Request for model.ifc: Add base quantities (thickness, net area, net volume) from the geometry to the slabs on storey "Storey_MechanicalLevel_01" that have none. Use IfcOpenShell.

First a look at what the model holds.

```python
import ifcopenshell
import ifcopenshell.util.element
import ifcopenshell.util.unit

model = ifcopenshell.open("model.ifc")
print(model.schema)
for unit_type in ("LENGTHUNIT", "AREAUNIT", "VOLUMEUNIT"):
    print(unit_type, ifcopenshell.util.unit.calculate_unit_scale(model, unit_type))
storey = next(s for s in model.by_type("IfcBuildingStorey") if s.Name == "Storey_MechanicalLevel_01")
slabs = [e for e in ifcopenshell.util.element.get_decomposition(storey) if e.is_a("IfcSlab")]
for e in sorted(slabs, key=lambda e: e.id()):
    print(e.id(), e.is_a(), e.Name, list(ifcopenshell.util.element.get_psets(e, qtos_only=True)), sep=" | ")
```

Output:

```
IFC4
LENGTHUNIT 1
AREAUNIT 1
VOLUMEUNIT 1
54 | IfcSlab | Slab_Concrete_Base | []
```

```python
import ifcopenshell
import ifcopenshell.api.pset
import ifcopenshell.geom
import ifcopenshell.util.element
import ifcopenshell.util.shape
import ifcopenshell.util.unit

model = ifcopenshell.open("model.ifc")
unit_scale = ifcopenshell.util.unit.calculate_unit_scale(model)
area_scale = ifcopenshell.util.unit.calculate_unit_scale(model, "AREAUNIT")
volume_scale = ifcopenshell.util.unit.calculate_unit_scale(model, "VOLUMEUNIT")
settings = ifcopenshell.geom.settings()

storey = next(s for s in model.by_type("IfcBuildingStorey") if s.Name == "Storey_MechanicalLevel_01")
slabs = [e for e in ifcopenshell.util.element.get_decomposition(storey) if e.is_a("IfcSlab")]

for e in sorted(slabs, key=lambda e: e.id()):
    if ifcopenshell.util.element.get_psets(e, qtos_only=True, should_inherit=False):
        continue
    # Geometry comes back in metres, in the element's own axes.
    shape = ifcopenshell.geom.create_shape(settings, e)
    values = {
        "Width": ifcopenshell.util.shape.get_z(shape.geometry) / unit_scale,
        "NetArea": ifcopenshell.util.shape.get_footprint_area(shape.geometry) / area_scale,
        "NetVolume": ifcopenshell.util.shape.get_volume(shape.geometry) / volume_scale,
    }
    qto = ifcopenshell.api.pset.add_qto(model, product=e, name="Qto_SlabBaseQuantities")
    ifcopenshell.api.pset.edit_qto(model, qto=qto, properties=values)
    print(e.id(), {k: round(v, 3) for k, v in values.items()})

model.write("model_rev.ifc")
```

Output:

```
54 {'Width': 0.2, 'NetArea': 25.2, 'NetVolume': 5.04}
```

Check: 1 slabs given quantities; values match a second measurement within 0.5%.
